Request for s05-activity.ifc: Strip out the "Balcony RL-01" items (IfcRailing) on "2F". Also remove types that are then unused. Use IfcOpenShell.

First a look at what the model holds.

```python
import ifcopenshell
import ifcopenshell.util.element

model = ifcopenshell.open("s05-activity.ifc")
print(model.schema)
storey = next(s for s in model.by_type("IfcBuildingStorey") if s.Name == "2F")
railings = [e for e in ifcopenshell.util.element.get_decomposition(storey) if e.is_a("IfcRailing")]
seen = {}
for e in railings:
    element_type = ifcopenshell.util.element.get_type(e)
    name = element_type.Name if element_type not in (None, e) else None
    seen[name] = seen.get(name, 0) + 1
for name, count in sorted(seen.items(), key=str):
    print(count, "x", name)
```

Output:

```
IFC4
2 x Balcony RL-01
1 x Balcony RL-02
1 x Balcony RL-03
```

```python
import ifcopenshell
import ifcopenshell.api.root
import ifcopenshell.util.element

model = ifcopenshell.open("s05-activity.ifc")

storey = next(s for s in model.by_type("IfcBuildingStorey") if s.Name == "2F")
railings = [e for e in ifcopenshell.util.element.get_decomposition(storey) if e.is_a("IfcRailing")]
targets = [e for e in railings if (t := ifcopenshell.util.element.get_type(e)) not in (None, e) and t.Name == "Balcony RL-01"]
types = {ifcopenshell.util.element.get_type(e) for e in targets} - {None, *targets}

for e in targets:
    ifcopenshell.api.root.remove_product(model, product=e)
print(len(targets), "removed")

unused = [t for t in types if not ifcopenshell.util.element.get_types(t)]
for t in unused:
    ifcopenshell.api.root.remove_product(model, product=t)
print(len(unused), "unused types removed")

model.write("s05-activity_rev.ifc")
```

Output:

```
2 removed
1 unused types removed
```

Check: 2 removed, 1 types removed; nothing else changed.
